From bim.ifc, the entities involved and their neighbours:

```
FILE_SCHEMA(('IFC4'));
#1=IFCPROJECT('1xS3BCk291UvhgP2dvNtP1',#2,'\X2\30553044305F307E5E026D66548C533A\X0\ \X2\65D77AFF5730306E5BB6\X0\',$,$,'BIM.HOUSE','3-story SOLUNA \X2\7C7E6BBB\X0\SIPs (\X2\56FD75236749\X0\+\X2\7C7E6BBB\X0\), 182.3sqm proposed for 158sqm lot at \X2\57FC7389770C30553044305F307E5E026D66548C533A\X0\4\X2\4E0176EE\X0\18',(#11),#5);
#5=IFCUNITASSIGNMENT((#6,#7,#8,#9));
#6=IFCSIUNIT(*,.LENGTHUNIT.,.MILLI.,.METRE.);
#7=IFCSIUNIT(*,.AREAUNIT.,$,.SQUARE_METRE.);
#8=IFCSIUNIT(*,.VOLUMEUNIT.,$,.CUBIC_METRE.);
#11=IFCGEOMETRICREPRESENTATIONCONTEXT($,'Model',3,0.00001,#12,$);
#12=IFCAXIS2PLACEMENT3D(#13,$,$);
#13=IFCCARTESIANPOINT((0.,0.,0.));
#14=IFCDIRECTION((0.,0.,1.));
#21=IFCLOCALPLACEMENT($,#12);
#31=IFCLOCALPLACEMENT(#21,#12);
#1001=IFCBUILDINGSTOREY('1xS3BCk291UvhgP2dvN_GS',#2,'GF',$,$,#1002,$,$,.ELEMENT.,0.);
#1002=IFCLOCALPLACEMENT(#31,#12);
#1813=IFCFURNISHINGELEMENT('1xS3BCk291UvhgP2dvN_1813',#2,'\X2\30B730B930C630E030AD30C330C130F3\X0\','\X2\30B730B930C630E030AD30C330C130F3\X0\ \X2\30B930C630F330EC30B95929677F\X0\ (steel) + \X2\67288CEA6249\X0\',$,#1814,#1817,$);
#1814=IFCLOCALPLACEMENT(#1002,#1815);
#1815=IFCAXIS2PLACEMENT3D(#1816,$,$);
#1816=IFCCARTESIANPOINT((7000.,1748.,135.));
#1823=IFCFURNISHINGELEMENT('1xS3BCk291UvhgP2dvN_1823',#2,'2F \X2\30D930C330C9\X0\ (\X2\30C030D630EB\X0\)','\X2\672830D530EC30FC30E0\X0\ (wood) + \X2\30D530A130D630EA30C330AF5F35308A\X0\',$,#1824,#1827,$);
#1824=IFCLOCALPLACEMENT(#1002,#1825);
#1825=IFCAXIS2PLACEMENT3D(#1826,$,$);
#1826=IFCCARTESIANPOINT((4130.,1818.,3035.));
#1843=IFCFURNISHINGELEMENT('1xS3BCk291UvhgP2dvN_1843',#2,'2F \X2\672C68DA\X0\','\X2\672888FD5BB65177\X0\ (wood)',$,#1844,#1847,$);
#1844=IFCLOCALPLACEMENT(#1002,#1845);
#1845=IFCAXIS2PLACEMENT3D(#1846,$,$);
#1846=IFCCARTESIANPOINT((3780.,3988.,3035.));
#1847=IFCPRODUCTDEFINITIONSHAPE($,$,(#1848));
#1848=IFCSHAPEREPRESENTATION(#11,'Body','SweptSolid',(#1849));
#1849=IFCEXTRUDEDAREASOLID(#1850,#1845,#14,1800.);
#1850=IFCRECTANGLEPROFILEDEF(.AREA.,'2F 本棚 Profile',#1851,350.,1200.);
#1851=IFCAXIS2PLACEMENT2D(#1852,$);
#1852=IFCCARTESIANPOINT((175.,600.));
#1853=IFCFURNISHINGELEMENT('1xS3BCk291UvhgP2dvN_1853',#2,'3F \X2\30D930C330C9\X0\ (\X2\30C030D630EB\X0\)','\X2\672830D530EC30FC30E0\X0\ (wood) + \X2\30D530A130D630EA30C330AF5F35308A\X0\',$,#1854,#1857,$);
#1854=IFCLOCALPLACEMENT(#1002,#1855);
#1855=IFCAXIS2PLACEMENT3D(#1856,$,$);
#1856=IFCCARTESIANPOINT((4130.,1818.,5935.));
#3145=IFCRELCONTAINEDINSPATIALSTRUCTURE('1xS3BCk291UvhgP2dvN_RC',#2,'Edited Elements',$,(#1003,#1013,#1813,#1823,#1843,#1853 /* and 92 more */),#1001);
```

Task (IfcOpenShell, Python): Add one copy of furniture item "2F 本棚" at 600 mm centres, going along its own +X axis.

```python
import ifcopenshell
import ifcopenshell.api.geometry
import ifcopenshell.api.root
import ifcopenshell.util.element
import ifcopenshell.util.placement
import ifcopenshell.util.unit

model = ifcopenshell.open("bim.ifc")
unit_scale = ifcopenshell.util.unit.calculate_unit_scale(model)


def reuse_history(source, copy):
    """copy_class also copies each property set's owner history, people and application; keep the originals."""
    for rel in copy.IsDefinedBy:
        if rel.is_a("IfcRelDefinesByProperties") and (history := rel.RelatingPropertyDefinition.OwnerHistory):
            rel.RelatingPropertyDefinition.OwnerHistory = source.OwnerHistory
            ifcopenshell.util.element.remove_deep2(model, history)


source = model.by_guid("1xS3BCk291UvhgP2dvN_1843")
base = ifcopenshell.util.placement.get_local_placement(source.ObjectPlacement)
step = base[:3, 0] * 0.6 / unit_scale

for i in range(1, 2):
    copy = ifcopenshell.api.root.copy_class(model, product=source)
    copy.Representation = ifcopenshell.util.element.copy_deep(
        model, source.Representation, exclude=["IfcGeometricRepresentationContext", "IfcRepresentationMap"]
    )
    reuse_history(source, copy)
    matrix = base.copy()
    matrix[:3, 3] += i * step
    print("added at", matrix[:3, 3].round(3) + 0.0)
    ifcopenshell.api.geometry.edit_object_placement(model, product=copy, matrix=matrix, is_si=False)

model.write("bim_v2.ifc")
```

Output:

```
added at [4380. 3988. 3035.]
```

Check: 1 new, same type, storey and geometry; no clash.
